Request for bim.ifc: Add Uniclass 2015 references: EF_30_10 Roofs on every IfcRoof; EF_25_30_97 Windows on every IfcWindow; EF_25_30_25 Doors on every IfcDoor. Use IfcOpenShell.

First a look at what the model holds.

```python
import ifcopenshell

model = ifcopenshell.open("bim.ifc")
print(model.schema)
print("classifications:", [c.Name for c in model.by_type("IfcClassification")])
for ifc_class in ("IfcDoor", "IfcRoof", "IfcStair", "IfcWall", "IfcWindow"):
    print(ifc_class, len(model.by_type(ifc_class)))
```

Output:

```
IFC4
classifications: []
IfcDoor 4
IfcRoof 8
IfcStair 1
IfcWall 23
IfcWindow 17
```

```python
import ifcopenshell
import ifcopenshell.api.classification

model = ifcopenshell.open("bim.ifc")

system = ifcopenshell.api.classification.add_classification(model, classification="Uniclass 2015")

codes = {
    "IfcRoof": ("EF_30_10", "Roofs"),
    "IfcWindow": ("EF_25_30_97", "Windows"),
    "IfcDoor": ("EF_25_30_25", "Doors"),
}
for ifc_class, (code, name) in codes.items():
    products = model.by_type(ifc_class)
    ifcopenshell.api.classification.add_reference(
        model, products=products, classification=system, identification=code, name=name
    )
    print(code, len(products))

model.write("bim_v2.ifc")
```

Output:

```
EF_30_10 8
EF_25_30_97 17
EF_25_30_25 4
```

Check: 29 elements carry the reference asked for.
